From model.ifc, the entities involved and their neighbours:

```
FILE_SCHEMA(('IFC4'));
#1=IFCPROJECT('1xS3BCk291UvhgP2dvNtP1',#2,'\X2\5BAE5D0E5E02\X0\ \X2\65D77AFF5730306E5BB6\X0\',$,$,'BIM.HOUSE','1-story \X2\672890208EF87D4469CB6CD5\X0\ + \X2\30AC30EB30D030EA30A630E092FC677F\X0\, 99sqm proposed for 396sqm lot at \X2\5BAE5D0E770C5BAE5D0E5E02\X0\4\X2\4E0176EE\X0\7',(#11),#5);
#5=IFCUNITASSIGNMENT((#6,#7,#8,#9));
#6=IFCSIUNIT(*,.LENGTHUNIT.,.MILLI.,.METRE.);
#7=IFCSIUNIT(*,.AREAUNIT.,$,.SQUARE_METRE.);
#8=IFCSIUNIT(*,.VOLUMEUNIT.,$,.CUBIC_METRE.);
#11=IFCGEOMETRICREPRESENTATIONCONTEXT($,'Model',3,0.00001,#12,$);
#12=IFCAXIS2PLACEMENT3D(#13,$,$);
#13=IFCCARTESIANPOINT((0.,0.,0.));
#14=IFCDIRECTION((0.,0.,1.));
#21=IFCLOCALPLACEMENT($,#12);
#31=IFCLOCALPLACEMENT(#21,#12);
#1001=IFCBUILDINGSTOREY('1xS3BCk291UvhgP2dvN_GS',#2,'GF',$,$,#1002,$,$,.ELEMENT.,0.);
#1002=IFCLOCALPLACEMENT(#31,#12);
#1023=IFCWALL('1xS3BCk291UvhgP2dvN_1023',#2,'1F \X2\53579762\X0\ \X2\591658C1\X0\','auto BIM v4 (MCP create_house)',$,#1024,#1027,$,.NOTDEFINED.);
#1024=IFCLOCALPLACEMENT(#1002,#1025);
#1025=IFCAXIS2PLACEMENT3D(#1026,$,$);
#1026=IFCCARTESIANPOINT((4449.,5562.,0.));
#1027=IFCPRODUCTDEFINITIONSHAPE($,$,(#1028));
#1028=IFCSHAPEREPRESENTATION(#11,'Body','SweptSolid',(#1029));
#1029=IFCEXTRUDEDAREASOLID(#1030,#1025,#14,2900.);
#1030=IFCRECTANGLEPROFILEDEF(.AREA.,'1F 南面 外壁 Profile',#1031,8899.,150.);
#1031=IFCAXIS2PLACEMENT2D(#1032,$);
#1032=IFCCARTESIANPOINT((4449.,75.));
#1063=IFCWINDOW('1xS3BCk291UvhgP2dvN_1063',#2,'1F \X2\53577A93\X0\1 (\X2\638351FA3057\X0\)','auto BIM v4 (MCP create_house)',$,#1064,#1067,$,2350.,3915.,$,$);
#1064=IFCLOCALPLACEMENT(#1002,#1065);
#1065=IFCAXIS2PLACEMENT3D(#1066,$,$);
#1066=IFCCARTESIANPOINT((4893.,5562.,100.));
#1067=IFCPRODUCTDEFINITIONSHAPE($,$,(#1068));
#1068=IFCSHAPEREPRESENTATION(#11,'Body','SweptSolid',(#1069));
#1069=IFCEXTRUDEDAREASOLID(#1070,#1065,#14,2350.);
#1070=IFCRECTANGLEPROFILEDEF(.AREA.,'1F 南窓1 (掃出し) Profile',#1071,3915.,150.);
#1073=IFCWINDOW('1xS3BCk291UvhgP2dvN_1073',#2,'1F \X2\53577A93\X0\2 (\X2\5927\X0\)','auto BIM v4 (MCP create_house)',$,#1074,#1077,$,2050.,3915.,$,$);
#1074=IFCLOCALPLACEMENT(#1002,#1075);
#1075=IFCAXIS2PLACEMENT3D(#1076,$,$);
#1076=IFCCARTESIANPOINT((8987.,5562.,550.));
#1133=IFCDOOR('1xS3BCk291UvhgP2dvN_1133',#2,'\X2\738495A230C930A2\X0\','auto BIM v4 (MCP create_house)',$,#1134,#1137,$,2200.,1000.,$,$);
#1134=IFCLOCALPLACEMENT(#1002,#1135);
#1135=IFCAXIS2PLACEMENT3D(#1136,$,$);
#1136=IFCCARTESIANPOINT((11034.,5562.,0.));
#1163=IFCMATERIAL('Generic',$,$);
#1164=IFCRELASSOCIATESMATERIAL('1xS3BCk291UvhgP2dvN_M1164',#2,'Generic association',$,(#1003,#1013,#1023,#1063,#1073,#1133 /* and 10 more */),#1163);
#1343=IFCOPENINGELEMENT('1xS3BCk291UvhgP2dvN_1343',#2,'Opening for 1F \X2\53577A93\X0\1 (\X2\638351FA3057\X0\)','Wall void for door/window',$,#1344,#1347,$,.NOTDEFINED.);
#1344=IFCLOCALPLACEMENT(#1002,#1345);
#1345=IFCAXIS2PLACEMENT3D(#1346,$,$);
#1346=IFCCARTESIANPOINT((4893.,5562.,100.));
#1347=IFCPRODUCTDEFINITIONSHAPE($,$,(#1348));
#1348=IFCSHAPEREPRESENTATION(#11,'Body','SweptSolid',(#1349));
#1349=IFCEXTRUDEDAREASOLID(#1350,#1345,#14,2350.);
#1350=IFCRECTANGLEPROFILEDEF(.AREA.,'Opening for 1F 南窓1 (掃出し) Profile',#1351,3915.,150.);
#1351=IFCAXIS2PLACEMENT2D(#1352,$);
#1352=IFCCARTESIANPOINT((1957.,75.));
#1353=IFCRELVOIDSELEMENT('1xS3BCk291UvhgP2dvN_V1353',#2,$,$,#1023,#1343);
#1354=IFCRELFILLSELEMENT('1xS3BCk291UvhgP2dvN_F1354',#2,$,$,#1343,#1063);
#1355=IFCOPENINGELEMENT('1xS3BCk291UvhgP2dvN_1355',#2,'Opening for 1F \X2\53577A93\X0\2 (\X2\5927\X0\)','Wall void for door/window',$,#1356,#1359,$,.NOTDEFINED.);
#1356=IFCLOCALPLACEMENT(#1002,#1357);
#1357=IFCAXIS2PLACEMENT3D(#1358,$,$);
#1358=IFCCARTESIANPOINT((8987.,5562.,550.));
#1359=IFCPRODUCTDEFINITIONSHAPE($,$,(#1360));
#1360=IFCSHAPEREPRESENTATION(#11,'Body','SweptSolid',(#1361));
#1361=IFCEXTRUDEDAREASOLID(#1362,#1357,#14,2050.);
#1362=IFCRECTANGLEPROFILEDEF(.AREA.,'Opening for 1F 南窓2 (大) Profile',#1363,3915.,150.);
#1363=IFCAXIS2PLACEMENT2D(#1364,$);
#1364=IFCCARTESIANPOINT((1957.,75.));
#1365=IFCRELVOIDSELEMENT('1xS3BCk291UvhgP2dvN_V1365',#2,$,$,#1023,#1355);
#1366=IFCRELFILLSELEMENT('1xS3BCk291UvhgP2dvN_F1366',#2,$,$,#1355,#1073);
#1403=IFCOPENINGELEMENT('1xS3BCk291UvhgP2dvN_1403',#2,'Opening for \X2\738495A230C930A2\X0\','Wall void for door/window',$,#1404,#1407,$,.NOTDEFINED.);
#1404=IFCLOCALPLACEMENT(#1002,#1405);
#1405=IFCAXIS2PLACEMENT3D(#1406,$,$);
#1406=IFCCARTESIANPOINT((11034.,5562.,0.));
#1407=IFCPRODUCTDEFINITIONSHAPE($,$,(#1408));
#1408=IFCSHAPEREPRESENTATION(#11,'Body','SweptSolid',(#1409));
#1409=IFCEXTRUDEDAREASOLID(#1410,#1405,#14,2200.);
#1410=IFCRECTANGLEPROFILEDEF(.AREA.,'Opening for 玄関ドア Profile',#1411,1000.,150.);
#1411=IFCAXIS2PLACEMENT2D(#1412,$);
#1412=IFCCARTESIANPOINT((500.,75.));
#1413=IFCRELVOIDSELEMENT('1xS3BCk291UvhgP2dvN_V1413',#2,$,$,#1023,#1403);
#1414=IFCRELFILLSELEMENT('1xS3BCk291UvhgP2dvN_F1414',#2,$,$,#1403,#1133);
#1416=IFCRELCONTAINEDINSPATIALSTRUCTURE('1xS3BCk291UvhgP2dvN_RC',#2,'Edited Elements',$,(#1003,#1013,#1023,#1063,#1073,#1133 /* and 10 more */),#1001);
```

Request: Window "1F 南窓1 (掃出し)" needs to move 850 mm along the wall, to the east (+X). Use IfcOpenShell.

```python
import ifcopenshell
import ifcopenshell.api.geometry
import ifcopenshell.util.placement
import ifcopenshell.util.unit

model = ifcopenshell.open("model.ifc")
unit_scale = ifcopenshell.util.unit.calculate_unit_scale(model)

window = model.by_guid("1xS3BCk291UvhgP2dvN_1063")
opening = window.FillsVoids[0].RelatingOpeningElement
wall = opening.VoidsElements[0].RelatingBuildingElement

wall_matrix = ifcopenshell.util.placement.get_local_placement(wall.ObjectPlacement)
shift = wall_matrix[:3, 0] * 0.85 / unit_scale
before = ifcopenshell.util.placement.get_local_placement(window.ObjectPlacement)[:3, 3].copy()

# The window is not placed relative to its opening, so move both.
for product in (opening, window):
    matrix = ifcopenshell.util.placement.get_local_placement(product.ObjectPlacement)
    matrix[:3, 3] += shift
    ifcopenshell.api.geometry.edit_object_placement(model, product=product, matrix=matrix, is_si=False)

after = ifcopenshell.util.placement.get_local_placement(window.ObjectPlacement)[:3, 3]
print("window moved by", (after - before).round(3) + 0.0)

model.write("model_v2.ifc")
```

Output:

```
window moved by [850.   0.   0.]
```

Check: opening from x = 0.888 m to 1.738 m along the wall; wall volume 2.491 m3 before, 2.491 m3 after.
